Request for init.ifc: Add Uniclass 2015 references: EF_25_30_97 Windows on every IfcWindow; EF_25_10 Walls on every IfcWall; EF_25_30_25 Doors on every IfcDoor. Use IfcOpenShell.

First a look at what the model holds.

```python
import ifcopenshell

model = ifcopenshell.open("init.ifc")
print(model.schema)
print("classifications:", [c.Name for c in model.by_type("IfcClassification")])
for ifc_class in ("IfcDoor", "IfcRoof", "IfcStair", "IfcWall", "IfcWindow"):
    print(ifc_class, len(model.by_type(ifc_class)))
```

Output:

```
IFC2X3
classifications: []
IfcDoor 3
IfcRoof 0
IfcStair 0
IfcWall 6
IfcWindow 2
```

```python
import ifcopenshell
import ifcopenshell.api.classification

model = ifcopenshell.open("init.ifc")

# IFC2X3 requires Source and Edition and has no link from the project to the system.
system = model.create_entity("IfcClassification", Source="NBS", Edition="2015", Name="Uniclass 2015")

codes = {
    "IfcWindow": ("EF_25_30_97", "Windows"),
    "IfcWall": ("EF_25_10", "Walls"),
    "IfcDoor": ("EF_25_30_25", "Doors"),
}
for ifc_class, (code, name) in codes.items():
    products = model.by_type(ifc_class)
    ifcopenshell.api.classification.add_reference(
        model, products=products, classification=system, identification=code, name=name
    )
    print(code, len(products))

model.write("init_v2.ifc")
```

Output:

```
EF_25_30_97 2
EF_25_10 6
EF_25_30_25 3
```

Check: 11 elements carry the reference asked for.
